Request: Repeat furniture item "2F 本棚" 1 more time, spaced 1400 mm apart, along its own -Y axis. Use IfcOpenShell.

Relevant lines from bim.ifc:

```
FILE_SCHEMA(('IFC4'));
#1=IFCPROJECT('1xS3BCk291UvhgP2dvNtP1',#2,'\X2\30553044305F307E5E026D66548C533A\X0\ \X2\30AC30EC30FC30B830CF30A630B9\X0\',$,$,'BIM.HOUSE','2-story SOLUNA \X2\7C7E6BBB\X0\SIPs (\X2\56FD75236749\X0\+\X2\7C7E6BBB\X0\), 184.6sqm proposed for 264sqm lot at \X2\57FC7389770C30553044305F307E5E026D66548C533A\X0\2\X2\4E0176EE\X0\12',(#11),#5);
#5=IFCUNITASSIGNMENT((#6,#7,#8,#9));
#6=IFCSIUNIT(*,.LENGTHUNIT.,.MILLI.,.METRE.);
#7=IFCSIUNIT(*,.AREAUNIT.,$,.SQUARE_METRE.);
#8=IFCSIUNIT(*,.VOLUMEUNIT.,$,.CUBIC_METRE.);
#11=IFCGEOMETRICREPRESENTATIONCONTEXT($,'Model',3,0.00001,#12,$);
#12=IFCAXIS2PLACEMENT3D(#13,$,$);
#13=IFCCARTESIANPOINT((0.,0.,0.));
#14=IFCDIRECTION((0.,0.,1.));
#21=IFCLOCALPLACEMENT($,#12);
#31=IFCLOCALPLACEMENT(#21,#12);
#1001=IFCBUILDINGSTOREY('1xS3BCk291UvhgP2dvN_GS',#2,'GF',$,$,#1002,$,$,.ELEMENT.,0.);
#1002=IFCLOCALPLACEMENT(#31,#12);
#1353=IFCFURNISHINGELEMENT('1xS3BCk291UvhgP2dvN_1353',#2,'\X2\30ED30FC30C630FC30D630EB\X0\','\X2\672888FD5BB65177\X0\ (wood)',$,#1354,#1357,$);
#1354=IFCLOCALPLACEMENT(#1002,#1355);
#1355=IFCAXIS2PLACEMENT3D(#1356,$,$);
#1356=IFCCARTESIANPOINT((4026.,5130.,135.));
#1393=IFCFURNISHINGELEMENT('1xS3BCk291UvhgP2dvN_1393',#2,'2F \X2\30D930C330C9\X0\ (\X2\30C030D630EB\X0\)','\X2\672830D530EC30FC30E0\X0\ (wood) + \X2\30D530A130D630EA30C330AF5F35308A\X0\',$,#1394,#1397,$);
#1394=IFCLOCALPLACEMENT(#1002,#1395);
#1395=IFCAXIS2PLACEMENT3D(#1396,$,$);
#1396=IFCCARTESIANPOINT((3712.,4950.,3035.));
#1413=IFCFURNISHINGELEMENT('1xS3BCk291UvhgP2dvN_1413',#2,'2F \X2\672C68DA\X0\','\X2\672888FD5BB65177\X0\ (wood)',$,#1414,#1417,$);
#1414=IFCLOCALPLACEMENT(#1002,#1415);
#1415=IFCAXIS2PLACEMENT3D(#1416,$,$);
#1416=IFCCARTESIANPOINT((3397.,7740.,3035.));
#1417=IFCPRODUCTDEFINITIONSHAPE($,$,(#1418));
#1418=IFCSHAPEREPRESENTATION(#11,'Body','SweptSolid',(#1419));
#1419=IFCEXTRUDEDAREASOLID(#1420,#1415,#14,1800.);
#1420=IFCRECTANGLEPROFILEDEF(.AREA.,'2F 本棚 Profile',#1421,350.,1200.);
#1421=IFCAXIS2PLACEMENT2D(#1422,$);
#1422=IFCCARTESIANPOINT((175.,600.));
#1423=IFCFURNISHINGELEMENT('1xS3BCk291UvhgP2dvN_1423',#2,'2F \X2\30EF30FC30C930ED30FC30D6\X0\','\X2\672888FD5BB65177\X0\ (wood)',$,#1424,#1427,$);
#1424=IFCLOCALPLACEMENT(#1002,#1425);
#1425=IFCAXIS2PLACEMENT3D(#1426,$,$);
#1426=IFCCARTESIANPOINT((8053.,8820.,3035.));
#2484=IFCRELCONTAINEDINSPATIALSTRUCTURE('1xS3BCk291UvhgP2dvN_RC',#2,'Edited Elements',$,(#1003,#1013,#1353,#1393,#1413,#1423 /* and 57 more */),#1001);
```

```python
import ifcopenshell
import ifcopenshell.api.geometry
import ifcopenshell.api.root
import ifcopenshell.util.element
import ifcopenshell.util.placement
import ifcopenshell.util.unit

model = ifcopenshell.open("bim.ifc")
unit_scale = ifcopenshell.util.unit.calculate_unit_scale(model)


def reuse_history(source, copy):
    """copy_class also copies each property set's owner history, people and application; keep the originals."""
    for rel in copy.IsDefinedBy:
        if rel.is_a("IfcRelDefinesByProperties") and (history := rel.RelatingPropertyDefinition.OwnerHistory):
            rel.RelatingPropertyDefinition.OwnerHistory = source.OwnerHistory
            ifcopenshell.util.element.remove_deep2(model, history)


source = model.by_id(1413)
base = ifcopenshell.util.placement.get_local_placement(source.ObjectPlacement)
step = -base[:3, 1] * 1.4 / unit_scale

for i in range(1, 2):
    copy = ifcopenshell.api.root.copy_class(model, product=source)
    copy.Representation = ifcopenshell.util.element.copy_deep(
        model, source.Representation, exclude=["IfcGeometricRepresentationContext", "IfcRepresentationMap"]
    )
    reuse_history(source, copy)
    matrix = base.copy()
    matrix[:3, 3] += i * step
    print("added at", matrix[:3, 3].round(3) + 0.0)
    ifcopenshell.api.geometry.edit_object_placement(model, product=copy, matrix=matrix, is_si=False)

model.write("bim_edited.ifc")
```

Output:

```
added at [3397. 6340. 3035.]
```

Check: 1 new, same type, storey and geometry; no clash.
